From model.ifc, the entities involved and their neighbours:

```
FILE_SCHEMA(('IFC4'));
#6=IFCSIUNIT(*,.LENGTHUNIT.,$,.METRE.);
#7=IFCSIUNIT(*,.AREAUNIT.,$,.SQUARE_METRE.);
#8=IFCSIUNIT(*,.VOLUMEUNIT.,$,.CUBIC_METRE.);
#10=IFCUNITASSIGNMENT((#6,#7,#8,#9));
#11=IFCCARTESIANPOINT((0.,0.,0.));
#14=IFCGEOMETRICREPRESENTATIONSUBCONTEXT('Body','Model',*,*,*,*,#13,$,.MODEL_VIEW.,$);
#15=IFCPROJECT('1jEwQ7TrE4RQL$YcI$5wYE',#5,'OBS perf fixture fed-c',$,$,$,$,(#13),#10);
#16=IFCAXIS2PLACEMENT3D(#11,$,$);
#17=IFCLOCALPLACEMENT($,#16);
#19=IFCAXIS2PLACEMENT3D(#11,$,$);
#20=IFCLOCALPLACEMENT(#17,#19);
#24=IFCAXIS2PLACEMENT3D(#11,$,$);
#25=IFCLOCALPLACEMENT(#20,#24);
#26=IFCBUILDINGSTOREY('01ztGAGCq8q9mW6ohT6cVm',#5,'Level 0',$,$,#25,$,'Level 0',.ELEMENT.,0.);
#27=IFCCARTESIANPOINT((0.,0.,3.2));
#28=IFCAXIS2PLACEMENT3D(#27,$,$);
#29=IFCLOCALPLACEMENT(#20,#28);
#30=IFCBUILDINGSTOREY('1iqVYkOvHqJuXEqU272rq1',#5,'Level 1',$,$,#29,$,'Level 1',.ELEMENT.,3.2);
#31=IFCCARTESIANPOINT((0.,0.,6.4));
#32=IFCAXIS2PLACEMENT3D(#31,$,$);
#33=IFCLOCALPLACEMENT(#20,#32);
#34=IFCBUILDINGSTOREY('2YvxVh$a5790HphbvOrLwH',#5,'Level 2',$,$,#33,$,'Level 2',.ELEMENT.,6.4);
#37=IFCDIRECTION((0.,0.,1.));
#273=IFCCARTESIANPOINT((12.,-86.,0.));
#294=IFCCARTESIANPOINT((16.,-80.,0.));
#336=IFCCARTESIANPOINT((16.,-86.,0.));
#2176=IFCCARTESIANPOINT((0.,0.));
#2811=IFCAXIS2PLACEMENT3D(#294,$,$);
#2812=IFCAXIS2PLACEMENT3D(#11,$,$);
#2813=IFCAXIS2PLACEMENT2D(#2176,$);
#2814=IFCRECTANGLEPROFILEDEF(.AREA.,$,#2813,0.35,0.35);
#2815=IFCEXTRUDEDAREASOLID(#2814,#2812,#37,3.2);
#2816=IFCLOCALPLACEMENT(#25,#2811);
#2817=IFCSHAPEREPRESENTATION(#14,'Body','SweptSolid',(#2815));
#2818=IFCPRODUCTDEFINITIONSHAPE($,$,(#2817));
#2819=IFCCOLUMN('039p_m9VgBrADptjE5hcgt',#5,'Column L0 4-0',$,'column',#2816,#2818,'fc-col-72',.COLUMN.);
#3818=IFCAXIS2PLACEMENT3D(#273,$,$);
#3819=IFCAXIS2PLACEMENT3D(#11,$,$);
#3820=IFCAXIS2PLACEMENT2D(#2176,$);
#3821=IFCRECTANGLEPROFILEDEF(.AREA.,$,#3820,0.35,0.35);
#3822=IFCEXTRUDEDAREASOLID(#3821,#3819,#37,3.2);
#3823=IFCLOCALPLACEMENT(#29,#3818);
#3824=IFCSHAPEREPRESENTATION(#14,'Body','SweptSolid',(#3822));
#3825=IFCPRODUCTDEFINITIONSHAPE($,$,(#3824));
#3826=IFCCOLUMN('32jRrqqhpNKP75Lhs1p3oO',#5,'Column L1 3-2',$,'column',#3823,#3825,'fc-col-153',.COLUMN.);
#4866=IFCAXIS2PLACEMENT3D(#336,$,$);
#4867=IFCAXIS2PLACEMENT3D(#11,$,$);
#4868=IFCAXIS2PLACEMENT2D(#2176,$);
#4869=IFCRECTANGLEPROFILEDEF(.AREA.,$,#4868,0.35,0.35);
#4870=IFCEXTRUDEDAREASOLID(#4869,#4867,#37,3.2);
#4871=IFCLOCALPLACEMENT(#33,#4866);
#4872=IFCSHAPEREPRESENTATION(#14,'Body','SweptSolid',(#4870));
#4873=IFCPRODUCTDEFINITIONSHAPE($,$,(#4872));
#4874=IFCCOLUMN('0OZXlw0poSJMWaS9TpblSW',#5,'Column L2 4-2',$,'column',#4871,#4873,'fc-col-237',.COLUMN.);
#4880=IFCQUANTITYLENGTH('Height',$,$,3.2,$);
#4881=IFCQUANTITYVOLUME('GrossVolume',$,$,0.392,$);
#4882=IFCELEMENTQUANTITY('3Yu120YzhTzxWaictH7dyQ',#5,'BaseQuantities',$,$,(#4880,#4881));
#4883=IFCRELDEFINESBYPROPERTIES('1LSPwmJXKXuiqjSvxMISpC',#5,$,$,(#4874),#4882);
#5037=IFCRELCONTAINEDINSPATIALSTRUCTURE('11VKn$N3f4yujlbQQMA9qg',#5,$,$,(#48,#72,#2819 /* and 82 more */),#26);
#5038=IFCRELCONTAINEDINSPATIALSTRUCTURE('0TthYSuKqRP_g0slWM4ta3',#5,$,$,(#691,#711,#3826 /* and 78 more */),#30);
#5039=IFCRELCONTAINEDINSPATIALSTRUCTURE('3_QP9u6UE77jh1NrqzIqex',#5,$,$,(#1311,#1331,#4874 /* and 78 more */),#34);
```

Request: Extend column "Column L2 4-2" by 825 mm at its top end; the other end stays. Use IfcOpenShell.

```python
import ifcopenshell
import ifcopenshell.api.pset
import ifcopenshell.util.element
import ifcopenshell.util.representation
import ifcopenshell.util.unit

model = ifcopenshell.open("model.ifc")
unit_scale = ifcopenshell.util.unit.calculate_unit_scale(model)

member = model.by_id(4874)
change = 0.825 / unit_scale

# The extrusion runs towards the end named, so only its depth changes.
body = ifcopenshell.util.representation.get_representation(member, "Model", "Body")
solid = body.Items[0]
old_length = solid.Depth
solid.Depth += change

# Update the stored length and volume.
qto = model.by_id(ifcopenshell.util.element.get_pset(member, "BaseQuantities", should_inherit=False)["id"])
ifcopenshell.api.pset.edit_qto(model, qto=qto, properties={
    "Height": solid.Depth,
    "GrossVolume": ifcopenshell.util.element.get_pset(member, "BaseQuantities", "GrossVolume") * solid.Depth / old_length,
})

print(f"length {old_length:g} -> {solid.Depth:g}")

model.write("model_v2.ifc")
```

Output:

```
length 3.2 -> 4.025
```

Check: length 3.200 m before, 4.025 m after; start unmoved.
